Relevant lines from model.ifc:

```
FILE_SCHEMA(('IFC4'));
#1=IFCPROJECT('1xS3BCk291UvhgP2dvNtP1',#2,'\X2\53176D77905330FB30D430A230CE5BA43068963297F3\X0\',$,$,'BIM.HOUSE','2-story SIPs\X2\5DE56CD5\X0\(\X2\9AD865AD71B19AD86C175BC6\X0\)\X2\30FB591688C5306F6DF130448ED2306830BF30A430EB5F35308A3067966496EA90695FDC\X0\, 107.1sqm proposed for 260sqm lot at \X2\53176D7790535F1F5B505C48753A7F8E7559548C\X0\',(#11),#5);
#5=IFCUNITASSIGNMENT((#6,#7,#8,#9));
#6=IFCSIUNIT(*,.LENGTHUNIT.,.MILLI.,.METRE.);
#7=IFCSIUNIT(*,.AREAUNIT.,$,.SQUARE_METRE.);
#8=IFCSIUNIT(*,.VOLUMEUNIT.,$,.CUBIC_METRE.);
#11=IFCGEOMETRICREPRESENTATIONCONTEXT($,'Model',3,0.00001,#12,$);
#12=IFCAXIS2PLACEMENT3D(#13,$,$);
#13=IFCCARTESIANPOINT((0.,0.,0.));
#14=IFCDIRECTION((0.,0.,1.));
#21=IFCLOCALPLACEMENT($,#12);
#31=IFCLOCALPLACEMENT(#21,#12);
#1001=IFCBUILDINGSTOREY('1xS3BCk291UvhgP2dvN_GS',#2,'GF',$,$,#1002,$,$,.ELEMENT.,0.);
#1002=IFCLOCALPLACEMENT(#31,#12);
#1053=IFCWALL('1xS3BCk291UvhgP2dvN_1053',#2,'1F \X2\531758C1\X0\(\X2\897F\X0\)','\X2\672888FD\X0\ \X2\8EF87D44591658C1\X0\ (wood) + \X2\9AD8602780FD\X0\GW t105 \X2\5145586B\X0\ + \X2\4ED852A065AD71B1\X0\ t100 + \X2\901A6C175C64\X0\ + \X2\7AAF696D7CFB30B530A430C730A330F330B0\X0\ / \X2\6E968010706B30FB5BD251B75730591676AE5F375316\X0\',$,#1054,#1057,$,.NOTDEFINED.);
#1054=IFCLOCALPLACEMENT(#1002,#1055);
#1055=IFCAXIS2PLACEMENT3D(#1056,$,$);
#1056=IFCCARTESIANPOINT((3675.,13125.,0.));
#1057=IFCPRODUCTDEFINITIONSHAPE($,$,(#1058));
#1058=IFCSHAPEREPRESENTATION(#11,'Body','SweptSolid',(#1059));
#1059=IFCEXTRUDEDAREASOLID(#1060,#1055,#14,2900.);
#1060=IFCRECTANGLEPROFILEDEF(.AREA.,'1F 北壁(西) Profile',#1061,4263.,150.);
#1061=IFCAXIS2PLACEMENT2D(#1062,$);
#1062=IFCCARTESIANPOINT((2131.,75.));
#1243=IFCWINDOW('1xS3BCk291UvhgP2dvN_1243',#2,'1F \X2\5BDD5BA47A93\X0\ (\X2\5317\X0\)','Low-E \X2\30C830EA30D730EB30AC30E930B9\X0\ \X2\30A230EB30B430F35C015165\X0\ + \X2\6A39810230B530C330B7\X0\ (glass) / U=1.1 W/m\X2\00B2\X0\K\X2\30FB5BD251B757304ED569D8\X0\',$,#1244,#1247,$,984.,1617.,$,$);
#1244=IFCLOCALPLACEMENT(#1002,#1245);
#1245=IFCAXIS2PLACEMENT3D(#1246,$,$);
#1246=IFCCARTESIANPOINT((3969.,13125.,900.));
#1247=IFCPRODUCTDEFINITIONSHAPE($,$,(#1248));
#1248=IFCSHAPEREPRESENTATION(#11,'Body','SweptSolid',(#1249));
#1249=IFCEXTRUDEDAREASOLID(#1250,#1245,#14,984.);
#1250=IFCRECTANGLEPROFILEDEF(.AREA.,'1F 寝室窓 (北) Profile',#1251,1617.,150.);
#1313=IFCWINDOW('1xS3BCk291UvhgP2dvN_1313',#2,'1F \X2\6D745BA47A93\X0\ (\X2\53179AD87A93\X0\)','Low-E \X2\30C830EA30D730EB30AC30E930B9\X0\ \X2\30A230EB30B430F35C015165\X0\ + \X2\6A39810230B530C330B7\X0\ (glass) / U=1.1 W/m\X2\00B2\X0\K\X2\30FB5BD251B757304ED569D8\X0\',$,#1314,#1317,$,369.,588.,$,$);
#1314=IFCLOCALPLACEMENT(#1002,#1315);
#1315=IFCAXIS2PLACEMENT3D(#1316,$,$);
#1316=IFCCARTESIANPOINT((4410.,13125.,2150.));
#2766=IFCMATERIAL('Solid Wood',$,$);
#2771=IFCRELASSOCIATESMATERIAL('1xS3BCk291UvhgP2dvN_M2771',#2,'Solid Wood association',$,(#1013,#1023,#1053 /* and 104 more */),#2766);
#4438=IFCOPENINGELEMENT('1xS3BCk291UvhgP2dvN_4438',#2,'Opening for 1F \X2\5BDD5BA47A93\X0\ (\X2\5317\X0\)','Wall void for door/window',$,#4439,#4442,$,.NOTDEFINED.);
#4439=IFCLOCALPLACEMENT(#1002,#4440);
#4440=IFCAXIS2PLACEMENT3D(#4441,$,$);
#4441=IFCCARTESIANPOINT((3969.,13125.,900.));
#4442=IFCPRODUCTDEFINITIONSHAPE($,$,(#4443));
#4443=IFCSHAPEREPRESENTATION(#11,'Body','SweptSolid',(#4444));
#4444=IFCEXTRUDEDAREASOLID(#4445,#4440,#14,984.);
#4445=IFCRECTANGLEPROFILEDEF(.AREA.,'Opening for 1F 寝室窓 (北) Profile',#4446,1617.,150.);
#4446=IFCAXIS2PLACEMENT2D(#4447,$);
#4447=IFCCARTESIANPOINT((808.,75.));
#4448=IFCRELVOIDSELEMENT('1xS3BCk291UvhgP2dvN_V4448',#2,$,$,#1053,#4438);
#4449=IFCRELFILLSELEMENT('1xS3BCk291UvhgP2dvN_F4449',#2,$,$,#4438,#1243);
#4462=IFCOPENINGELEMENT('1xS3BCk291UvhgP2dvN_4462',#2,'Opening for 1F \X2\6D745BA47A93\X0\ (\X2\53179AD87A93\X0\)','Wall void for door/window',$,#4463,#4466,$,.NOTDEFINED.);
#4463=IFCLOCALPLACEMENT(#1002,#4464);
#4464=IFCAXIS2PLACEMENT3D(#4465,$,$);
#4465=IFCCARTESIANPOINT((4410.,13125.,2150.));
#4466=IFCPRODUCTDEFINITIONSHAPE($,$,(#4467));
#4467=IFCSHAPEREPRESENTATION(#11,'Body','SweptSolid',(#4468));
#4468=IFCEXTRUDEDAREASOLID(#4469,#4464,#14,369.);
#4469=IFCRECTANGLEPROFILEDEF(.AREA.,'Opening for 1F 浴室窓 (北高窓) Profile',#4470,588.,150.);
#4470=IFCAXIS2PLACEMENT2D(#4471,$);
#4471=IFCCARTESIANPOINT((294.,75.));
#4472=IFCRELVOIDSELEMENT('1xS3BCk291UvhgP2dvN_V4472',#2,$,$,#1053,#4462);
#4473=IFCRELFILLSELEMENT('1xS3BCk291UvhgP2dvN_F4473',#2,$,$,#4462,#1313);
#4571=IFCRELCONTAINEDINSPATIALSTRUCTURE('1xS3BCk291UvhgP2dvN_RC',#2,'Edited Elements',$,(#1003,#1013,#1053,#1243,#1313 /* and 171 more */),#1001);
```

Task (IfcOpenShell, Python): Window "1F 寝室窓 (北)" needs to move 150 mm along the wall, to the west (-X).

```python
import ifcopenshell
import ifcopenshell.api.geometry
import ifcopenshell.util.placement

model = ifcopenshell.open("model.ifc")

window = model.by_guid("1xS3BCk291UvhgP2dvN_1243")
opening = window.FillsVoids[0].RelatingOpeningElement
wall = opening.VoidsElements[0].RelatingBuildingElement

wall_matrix = ifcopenshell.util.placement.get_local_placement(wall.ObjectPlacement)
shift = wall_matrix[:3, 0] * -150.0
before = ifcopenshell.util.placement.get_local_placement(window.ObjectPlacement)[:3, 3].copy()

# The window is not placed relative to its opening, so move both.
for product in (opening, window):
    matrix = ifcopenshell.util.placement.get_local_placement(product.ObjectPlacement)
    matrix[:3, 3] += shift
    ifcopenshell.api.geometry.edit_object_placement(model, product=product, matrix=matrix, is_si=False)

after = ifcopenshell.util.placement.get_local_placement(window.ObjectPlacement)[:3, 3]
print("window moved by", (after - before).round(3) + 0.0)

model.write("model-out.ifc")
```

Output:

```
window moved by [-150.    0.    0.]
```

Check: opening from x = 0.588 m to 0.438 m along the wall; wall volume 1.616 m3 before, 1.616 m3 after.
